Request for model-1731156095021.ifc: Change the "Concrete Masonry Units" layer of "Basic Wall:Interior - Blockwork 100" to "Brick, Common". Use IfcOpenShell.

First a look at what the model holds.

```python
import ifcopenshell
import ifcopenshell.util.element

model = ifcopenshell.open("model-1731156095021.ifc")
print(model.schema)
for layer_set in model.by_type("IfcMaterialLayerSet"):
    if layer_set.LayerSetName == "Basic Wall:Interior - Blockwork 100":
        for layer in layer_set.MaterialLayers:
            print(layer.id(), layer.Material and layer.Material.Name, layer.LayerThickness, sep=" | ")
        print(len(ifcopenshell.util.element.get_elements_by_material(model, layer_set)), "elements and types use it")
print(sorted(m.Name for m in model.by_type("IfcMaterial") if m.Name)[:60])
```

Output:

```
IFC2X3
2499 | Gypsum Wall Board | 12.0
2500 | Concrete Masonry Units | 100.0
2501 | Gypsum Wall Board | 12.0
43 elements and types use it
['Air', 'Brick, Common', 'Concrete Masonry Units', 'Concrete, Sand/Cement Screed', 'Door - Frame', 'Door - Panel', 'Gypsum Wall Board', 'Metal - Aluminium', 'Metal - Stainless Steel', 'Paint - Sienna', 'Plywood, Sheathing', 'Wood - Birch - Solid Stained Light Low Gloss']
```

```python
import ifcopenshell
import ifcopenshell.api.material

model = ifcopenshell.open("model-1731156095021.ifc")

layer_set = next(s for s in model.by_type("IfcMaterialLayerSet") if s.LayerSetName == "Basic Wall:Interior - Blockwork 100")
layer = next(l for l in layer_set.MaterialLayers if l.Material and l.Material.Name == "Concrete Masonry Units")
material = next(m for m in model.by_type("IfcMaterial") if m.Name == "Brick, Common")

# Point this one layer at the other material; renaming the old one would change it everywhere.
ifcopenshell.api.material.edit_layer(model, layer=layer, attributes={}, material=material)

print([l.Material.Name if l.Material else None for l in layer_set.MaterialLayers])

model.write("model-1731156095021_updated.ifc")
```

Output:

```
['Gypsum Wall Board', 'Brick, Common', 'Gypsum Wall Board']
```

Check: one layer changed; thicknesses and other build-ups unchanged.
